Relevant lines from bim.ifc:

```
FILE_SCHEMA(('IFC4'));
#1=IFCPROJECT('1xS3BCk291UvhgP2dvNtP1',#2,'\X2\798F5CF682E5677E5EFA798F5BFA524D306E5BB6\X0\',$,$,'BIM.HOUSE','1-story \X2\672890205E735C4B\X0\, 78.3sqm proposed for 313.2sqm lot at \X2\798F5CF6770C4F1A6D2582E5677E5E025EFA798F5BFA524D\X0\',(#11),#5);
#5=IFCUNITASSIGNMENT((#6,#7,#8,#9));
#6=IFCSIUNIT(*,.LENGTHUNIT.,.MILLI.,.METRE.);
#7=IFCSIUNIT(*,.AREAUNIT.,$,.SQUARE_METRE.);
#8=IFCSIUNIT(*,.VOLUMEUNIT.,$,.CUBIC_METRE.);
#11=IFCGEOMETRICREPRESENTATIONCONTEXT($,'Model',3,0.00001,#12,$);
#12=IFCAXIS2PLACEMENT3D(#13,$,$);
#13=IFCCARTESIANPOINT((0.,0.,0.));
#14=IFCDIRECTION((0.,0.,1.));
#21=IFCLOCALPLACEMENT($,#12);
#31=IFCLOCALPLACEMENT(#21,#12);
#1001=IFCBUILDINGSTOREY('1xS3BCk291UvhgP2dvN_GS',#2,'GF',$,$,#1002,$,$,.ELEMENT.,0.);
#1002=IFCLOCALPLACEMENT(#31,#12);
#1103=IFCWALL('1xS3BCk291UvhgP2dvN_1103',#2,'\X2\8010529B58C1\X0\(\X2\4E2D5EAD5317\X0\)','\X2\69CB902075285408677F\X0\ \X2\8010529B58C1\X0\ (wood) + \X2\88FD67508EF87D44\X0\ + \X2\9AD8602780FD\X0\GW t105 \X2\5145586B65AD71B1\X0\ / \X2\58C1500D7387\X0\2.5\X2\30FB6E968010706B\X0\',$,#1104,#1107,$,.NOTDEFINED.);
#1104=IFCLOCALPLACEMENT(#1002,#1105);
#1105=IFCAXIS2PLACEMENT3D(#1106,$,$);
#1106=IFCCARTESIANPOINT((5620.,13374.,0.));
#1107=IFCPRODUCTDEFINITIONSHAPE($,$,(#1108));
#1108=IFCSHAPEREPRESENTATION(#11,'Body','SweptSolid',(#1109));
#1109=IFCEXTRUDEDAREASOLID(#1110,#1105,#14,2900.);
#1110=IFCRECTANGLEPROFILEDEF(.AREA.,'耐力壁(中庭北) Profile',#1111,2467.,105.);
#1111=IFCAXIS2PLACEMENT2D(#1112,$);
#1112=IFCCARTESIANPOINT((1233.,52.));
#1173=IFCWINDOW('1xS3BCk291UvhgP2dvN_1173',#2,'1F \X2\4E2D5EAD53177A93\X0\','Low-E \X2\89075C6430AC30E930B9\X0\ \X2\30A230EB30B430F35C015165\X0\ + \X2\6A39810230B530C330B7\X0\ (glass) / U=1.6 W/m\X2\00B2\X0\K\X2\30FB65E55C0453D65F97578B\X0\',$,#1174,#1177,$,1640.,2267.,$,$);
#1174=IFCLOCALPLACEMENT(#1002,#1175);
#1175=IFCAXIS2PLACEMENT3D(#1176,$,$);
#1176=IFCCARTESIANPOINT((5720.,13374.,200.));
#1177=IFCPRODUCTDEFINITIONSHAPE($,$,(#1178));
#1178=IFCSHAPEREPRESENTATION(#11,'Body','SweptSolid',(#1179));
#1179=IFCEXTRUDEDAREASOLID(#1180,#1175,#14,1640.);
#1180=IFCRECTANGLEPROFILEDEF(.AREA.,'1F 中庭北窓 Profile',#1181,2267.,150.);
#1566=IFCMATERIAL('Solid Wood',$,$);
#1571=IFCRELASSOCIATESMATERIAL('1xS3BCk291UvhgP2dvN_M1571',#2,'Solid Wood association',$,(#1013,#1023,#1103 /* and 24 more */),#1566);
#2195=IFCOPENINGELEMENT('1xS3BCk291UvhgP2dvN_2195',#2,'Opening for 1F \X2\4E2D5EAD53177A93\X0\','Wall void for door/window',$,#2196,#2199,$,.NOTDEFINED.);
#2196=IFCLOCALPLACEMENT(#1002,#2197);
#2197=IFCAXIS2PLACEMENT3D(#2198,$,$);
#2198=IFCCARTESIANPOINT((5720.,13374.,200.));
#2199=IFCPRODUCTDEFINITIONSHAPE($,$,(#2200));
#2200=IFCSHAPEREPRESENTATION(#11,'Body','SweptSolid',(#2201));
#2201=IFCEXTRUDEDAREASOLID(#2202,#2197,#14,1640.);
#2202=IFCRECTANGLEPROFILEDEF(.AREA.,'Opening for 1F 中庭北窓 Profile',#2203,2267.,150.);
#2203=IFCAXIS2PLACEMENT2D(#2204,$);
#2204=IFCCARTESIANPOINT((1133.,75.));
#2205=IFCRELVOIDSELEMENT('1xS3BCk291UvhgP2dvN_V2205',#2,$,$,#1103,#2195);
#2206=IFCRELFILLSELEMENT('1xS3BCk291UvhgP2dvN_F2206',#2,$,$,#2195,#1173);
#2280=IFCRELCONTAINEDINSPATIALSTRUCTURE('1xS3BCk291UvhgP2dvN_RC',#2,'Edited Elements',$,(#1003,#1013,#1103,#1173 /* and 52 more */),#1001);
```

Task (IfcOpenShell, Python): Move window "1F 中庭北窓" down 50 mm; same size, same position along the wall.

```python
import numpy as np
import ifcopenshell
import ifcopenshell.api.geometry
import ifcopenshell.util.placement
import ifcopenshell.util.unit

model = ifcopenshell.open("bim.ifc")
unit_scale = ifcopenshell.util.unit.calculate_unit_scale(model)

window = model.by_id(1173)
opening = window.FillsVoids[0].RelatingOpeningElement
dz = -50.0

shift = np.array([0.0, 0.0, dz])
# The window is not placed relative to its opening, so move both.
for product in (opening, window):
    matrix = ifcopenshell.util.placement.get_local_placement(product.ObjectPlacement)
    matrix[:3, 3] += shift
    ifcopenshell.api.geometry.edit_object_placement(model, product=product, matrix=matrix, is_si=False)

print(f"moved by {dz * unit_scale:+.3f} m")

model.write("bim_updated.ifc")
```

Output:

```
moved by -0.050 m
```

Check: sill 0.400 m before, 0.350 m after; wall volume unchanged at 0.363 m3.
